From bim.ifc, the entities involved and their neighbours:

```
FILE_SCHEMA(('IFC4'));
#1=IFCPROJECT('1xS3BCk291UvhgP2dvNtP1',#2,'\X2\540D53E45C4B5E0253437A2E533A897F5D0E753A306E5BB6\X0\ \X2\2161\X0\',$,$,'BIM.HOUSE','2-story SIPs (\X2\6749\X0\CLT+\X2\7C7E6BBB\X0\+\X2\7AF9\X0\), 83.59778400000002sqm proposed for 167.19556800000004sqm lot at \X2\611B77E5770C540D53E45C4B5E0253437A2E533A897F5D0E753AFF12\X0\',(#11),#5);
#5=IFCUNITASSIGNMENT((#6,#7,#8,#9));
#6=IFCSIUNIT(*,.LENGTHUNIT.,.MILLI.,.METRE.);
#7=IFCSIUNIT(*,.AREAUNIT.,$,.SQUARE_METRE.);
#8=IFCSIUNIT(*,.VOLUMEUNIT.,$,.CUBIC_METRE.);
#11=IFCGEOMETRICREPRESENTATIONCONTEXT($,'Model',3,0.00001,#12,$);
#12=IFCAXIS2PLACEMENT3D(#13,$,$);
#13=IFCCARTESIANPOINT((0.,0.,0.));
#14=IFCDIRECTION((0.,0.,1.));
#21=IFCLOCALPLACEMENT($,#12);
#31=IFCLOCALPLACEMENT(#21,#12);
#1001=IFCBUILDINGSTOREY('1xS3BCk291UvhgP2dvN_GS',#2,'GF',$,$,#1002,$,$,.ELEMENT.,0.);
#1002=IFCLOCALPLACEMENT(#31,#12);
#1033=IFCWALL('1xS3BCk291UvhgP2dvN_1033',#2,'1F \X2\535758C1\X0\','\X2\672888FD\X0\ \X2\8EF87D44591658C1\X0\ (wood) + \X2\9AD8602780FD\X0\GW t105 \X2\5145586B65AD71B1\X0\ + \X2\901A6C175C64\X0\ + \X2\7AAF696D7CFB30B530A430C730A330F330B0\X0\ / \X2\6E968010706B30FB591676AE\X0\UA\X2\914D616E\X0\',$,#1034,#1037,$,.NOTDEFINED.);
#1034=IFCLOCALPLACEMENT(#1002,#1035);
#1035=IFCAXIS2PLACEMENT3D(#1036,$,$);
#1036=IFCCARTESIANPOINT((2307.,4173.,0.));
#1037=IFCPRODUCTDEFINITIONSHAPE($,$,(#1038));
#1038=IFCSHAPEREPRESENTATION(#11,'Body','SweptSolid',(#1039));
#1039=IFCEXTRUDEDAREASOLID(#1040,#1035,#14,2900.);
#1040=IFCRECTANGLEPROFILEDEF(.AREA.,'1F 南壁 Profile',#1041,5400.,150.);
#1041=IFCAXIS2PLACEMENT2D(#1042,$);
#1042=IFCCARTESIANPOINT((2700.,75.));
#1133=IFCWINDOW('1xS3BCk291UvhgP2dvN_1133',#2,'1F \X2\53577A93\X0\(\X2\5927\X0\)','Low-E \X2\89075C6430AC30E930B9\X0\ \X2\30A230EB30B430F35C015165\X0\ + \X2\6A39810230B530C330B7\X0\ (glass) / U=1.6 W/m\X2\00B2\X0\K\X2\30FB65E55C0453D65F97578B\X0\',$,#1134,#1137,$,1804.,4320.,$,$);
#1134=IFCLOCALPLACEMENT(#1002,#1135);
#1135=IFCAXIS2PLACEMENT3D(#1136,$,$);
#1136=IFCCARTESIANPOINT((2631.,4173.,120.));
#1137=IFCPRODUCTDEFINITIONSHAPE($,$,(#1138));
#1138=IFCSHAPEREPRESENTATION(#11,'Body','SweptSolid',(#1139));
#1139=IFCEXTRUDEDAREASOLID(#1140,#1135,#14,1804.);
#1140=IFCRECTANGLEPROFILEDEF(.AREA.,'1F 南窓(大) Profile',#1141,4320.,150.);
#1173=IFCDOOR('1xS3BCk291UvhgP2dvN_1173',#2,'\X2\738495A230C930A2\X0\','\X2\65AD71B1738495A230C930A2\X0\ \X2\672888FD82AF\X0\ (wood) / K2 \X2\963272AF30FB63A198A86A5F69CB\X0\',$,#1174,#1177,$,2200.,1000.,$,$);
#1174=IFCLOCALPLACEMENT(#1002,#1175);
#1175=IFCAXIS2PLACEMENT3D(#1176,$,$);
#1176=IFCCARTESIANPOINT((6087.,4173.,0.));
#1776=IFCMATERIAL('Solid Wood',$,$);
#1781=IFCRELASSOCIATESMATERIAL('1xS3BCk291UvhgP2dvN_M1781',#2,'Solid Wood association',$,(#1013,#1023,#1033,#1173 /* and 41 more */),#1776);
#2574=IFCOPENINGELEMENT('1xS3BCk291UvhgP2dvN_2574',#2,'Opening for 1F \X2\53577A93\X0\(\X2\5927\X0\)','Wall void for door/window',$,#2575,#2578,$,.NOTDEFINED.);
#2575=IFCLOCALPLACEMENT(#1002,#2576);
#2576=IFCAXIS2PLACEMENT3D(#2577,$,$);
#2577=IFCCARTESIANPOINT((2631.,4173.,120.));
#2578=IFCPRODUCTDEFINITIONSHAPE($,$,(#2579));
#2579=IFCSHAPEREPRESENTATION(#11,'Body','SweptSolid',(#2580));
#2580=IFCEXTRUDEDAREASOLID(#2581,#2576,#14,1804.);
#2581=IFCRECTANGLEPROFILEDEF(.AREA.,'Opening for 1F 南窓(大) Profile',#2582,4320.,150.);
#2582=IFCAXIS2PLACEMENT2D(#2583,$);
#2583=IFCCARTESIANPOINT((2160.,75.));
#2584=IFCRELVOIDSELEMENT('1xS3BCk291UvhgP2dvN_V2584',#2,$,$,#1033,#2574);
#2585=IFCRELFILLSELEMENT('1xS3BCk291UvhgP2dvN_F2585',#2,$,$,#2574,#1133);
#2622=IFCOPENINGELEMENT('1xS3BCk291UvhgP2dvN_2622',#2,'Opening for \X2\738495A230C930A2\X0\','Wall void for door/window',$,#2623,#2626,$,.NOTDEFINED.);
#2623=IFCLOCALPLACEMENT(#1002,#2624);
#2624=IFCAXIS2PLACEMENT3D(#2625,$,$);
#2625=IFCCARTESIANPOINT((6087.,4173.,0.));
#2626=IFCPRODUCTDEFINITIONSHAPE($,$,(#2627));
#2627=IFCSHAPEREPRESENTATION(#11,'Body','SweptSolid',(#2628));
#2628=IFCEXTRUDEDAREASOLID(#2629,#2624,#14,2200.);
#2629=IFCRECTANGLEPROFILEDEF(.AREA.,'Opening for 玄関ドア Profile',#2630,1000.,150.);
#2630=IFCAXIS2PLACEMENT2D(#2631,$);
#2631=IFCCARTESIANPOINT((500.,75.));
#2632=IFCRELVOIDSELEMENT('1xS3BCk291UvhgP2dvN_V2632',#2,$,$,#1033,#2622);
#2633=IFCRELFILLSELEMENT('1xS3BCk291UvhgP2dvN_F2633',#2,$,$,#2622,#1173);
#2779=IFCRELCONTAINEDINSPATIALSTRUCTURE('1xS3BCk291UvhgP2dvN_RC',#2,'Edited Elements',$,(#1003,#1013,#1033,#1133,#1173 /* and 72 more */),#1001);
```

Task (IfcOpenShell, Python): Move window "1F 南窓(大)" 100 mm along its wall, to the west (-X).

```python
import ifcopenshell
import ifcopenshell.api.geometry
import ifcopenshell.util.placement
import ifcopenshell.util.unit

model = ifcopenshell.open("bim.ifc")
unit_scale = ifcopenshell.util.unit.calculate_unit_scale(model)

window = model.by_id(1133)
opening = window.FillsVoids[0].RelatingOpeningElement
wall = opening.VoidsElements[0].RelatingBuildingElement

wall_matrix = ifcopenshell.util.placement.get_local_placement(wall.ObjectPlacement)
shift = wall_matrix[:3, 0] * -0.1 / unit_scale
before = ifcopenshell.util.placement.get_local_placement(window.ObjectPlacement)[:3, 3].copy()

# The window is not placed relative to its opening, so move both.
for product in (opening, window):
    matrix = ifcopenshell.util.placement.get_local_placement(product.ObjectPlacement)
    matrix[:3, 3] += shift
    ifcopenshell.api.geometry.edit_object_placement(model, product=product, matrix=matrix, is_si=False)

after = ifcopenshell.util.placement.get_local_placement(window.ObjectPlacement)[:3, 3]
print("window moved by", (after - before).round(3) + 0.0)

model.write("bim_v2.ifc")
```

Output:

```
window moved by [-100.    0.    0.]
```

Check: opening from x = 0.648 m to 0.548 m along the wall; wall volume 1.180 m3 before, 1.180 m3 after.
